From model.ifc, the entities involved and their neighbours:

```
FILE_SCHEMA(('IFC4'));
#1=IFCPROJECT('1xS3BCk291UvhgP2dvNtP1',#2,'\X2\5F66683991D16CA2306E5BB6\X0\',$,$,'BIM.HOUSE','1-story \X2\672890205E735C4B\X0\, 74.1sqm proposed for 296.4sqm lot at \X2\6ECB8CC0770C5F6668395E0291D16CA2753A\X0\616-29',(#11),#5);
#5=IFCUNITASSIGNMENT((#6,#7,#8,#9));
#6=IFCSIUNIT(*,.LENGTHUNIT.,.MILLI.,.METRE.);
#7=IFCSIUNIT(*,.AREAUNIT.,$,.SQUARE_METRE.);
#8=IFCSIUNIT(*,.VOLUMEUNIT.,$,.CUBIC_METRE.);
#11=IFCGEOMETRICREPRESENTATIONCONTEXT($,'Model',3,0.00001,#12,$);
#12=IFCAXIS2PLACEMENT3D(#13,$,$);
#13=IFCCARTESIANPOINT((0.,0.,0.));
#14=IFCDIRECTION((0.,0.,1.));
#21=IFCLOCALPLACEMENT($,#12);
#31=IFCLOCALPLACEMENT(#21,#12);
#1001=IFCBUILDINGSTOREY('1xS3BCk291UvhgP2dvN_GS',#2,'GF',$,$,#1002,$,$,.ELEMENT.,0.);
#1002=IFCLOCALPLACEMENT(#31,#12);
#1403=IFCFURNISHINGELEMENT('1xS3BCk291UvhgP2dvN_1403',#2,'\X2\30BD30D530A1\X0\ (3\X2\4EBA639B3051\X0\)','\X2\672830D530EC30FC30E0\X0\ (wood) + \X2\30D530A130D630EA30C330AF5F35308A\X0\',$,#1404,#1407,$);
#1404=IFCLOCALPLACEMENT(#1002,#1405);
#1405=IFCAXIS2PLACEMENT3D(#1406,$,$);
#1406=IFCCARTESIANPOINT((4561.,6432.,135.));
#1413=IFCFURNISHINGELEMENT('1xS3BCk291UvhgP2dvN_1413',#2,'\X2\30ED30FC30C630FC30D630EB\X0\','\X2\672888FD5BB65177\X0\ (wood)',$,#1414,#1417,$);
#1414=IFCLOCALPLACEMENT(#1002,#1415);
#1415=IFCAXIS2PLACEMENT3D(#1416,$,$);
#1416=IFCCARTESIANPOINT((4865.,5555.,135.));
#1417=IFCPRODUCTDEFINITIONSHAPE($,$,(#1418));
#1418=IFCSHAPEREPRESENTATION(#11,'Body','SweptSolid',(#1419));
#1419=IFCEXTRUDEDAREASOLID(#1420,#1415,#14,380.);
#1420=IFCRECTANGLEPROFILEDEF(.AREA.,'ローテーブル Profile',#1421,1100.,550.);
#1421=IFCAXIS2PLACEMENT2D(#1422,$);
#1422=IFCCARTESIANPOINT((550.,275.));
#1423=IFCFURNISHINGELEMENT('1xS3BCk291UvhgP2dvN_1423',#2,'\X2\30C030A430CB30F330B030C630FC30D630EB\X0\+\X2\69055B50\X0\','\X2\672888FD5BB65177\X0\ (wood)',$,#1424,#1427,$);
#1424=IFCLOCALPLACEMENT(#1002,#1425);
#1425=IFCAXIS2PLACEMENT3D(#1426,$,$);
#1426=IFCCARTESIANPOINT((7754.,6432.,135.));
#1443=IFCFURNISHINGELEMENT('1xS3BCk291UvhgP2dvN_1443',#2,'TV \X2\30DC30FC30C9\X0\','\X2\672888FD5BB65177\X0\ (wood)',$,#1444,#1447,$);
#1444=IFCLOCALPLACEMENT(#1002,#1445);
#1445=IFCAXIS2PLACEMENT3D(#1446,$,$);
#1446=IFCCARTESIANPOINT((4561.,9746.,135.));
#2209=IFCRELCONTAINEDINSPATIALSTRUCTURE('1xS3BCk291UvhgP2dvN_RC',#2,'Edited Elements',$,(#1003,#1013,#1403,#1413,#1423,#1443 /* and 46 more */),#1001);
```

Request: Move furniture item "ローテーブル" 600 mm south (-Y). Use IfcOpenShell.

```python
import ifcopenshell
import ifcopenshell.api.geometry
import ifcopenshell.util.placement
import ifcopenshell.util.unit

model = ifcopenshell.open("model.ifc")
unit_scale = ifcopenshell.util.unit.calculate_unit_scale(model)

item = model.by_guid("1xS3BCk291UvhgP2dvN_1413")
matrix = ifcopenshell.util.placement.get_local_placement(item.ObjectPlacement)
matrix[1, 3] -= 0.6 / unit_scale
ifcopenshell.api.geometry.edit_object_placement(model, product=item, matrix=matrix, is_si=False)

print(ifcopenshell.util.placement.get_local_placement(item.ObjectPlacement).round(3) + 0.0)

model.write("model-out.ifc")
```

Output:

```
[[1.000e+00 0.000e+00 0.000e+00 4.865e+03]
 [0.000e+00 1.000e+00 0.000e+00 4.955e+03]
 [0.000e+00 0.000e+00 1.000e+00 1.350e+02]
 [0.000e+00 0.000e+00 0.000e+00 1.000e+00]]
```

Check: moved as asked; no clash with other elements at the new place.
